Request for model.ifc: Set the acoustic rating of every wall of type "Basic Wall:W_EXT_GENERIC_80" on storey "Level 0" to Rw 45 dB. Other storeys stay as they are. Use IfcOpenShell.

First a look at what the model holds.

```python
import ifcopenshell
import ifcopenshell.util.element

model = ifcopenshell.open("model.ifc")
print(model.schema)
storey = next(s for s in model.by_type("IfcBuildingStorey") if s.Name == "Level 0")
walls = [e for e in ifcopenshell.util.element.get_decomposition(storey) if e.is_a("IfcWall")]
seen = {}
for e in walls:
    element_type = ifcopenshell.util.element.get_type(e)
    key = (element_type.Name if element_type != e and element_type else None, ifcopenshell.util.element.get_pset(e, "Pset_WallCommon", "AcousticRating"))
    seen[key] = seen.get(key, 0) + 1
for (name, value), count in sorted(seen.items(), key=str):
    print(count, "x", name, "|", value)
```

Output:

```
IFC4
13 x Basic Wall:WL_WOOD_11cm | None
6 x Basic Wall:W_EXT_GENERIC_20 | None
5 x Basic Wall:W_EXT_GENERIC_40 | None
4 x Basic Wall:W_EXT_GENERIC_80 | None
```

```python
import ifcopenshell
import ifcopenshell.api.pset
import ifcopenshell.util.element

model = ifcopenshell.open("model.ifc")

storey = next(s for s in model.by_type("IfcBuildingStorey") if s.Name == "Level 0")
walls = [e for e in ifcopenshell.util.element.get_decomposition(storey) if e.is_a("IfcWall")]

count = 0
for e in walls:
    element_type = ifcopenshell.util.element.get_type(e)
    if element_type in (None, e) or element_type.Name != "Basic Wall:W_EXT_GENERIC_80":
        continue
    # add_pset returns the element's existing set when there is one.
    pset = ifcopenshell.api.pset.add_pset(model, product=e, name="Pset_WallCommon")
    ifcopenshell.api.pset.edit_pset(model, pset=pset, properties={"AcousticRating": "Rw 45 dB"})
    count += 1

print(count, "walls updated")

model.write("model_edited.ifc")
```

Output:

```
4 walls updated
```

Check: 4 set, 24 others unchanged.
